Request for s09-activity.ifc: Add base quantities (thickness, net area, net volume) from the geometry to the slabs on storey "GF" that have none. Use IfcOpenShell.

First a look at what the model holds.

```python
import ifcopenshell
import ifcopenshell.util.element
import ifcopenshell.util.unit

model = ifcopenshell.open("s09-activity.ifc")
print(model.schema)
for unit_type in ("LENGTHUNIT", "AREAUNIT", "VOLUMEUNIT"):
    print(unit_type, ifcopenshell.util.unit.calculate_unit_scale(model, unit_type))
storey = next(s for s in model.by_type("IfcBuildingStorey") if s.Name == "GF")
slabs = [e for e in ifcopenshell.util.element.get_decomposition(storey) if e.is_a("IfcSlab")]
for e in sorted(slabs, key=lambda e: e.id()):
    print(e.id(), e.is_a(), e.Name, list(ifcopenshell.util.element.get_psets(e, qtos_only=True)), sep=" | ")
```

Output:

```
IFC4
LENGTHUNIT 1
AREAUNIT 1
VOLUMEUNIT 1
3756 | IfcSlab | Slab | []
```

```python
import ifcopenshell
import ifcopenshell.api.pset
import ifcopenshell.geom
import ifcopenshell.util.element
import ifcopenshell.util.shape
import ifcopenshell.util.unit

model = ifcopenshell.open("s09-activity.ifc")
unit_scale = ifcopenshell.util.unit.calculate_unit_scale(model)
area_scale = ifcopenshell.util.unit.calculate_unit_scale(model, "AREAUNIT")
volume_scale = ifcopenshell.util.unit.calculate_unit_scale(model, "VOLUMEUNIT")
settings = ifcopenshell.geom.settings()

storey = next(s for s in model.by_type("IfcBuildingStorey") if s.Name == "GF")
slabs = [e for e in ifcopenshell.util.element.get_decomposition(storey) if e.is_a("IfcSlab")]

for e in sorted(slabs, key=lambda e: e.id()):
    if ifcopenshell.util.element.get_psets(e, qtos_only=True, should_inherit=False):
        continue
    # Geometry comes back in metres, in the element's own axes.
    shape = ifcopenshell.geom.create_shape(settings, e)
    values = {
        "Width": ifcopenshell.util.shape.get_z(shape.geometry) / unit_scale,
        "NetArea": ifcopenshell.util.shape.get_footprint_area(shape.geometry) / area_scale,
        "NetVolume": ifcopenshell.util.shape.get_volume(shape.geometry) / volume_scale,
    }
    qto = ifcopenshell.api.pset.add_qto(model, product=e, name="Qto_SlabBaseQuantities")
    ifcopenshell.api.pset.edit_qto(model, qto=qto, properties=values)
    print(e.id(), {k: round(v, 3) for k, v in values.items()})

model.write("s09-activity_edited.ifc")
```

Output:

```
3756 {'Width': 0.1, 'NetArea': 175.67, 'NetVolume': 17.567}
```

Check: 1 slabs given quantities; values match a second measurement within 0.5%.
